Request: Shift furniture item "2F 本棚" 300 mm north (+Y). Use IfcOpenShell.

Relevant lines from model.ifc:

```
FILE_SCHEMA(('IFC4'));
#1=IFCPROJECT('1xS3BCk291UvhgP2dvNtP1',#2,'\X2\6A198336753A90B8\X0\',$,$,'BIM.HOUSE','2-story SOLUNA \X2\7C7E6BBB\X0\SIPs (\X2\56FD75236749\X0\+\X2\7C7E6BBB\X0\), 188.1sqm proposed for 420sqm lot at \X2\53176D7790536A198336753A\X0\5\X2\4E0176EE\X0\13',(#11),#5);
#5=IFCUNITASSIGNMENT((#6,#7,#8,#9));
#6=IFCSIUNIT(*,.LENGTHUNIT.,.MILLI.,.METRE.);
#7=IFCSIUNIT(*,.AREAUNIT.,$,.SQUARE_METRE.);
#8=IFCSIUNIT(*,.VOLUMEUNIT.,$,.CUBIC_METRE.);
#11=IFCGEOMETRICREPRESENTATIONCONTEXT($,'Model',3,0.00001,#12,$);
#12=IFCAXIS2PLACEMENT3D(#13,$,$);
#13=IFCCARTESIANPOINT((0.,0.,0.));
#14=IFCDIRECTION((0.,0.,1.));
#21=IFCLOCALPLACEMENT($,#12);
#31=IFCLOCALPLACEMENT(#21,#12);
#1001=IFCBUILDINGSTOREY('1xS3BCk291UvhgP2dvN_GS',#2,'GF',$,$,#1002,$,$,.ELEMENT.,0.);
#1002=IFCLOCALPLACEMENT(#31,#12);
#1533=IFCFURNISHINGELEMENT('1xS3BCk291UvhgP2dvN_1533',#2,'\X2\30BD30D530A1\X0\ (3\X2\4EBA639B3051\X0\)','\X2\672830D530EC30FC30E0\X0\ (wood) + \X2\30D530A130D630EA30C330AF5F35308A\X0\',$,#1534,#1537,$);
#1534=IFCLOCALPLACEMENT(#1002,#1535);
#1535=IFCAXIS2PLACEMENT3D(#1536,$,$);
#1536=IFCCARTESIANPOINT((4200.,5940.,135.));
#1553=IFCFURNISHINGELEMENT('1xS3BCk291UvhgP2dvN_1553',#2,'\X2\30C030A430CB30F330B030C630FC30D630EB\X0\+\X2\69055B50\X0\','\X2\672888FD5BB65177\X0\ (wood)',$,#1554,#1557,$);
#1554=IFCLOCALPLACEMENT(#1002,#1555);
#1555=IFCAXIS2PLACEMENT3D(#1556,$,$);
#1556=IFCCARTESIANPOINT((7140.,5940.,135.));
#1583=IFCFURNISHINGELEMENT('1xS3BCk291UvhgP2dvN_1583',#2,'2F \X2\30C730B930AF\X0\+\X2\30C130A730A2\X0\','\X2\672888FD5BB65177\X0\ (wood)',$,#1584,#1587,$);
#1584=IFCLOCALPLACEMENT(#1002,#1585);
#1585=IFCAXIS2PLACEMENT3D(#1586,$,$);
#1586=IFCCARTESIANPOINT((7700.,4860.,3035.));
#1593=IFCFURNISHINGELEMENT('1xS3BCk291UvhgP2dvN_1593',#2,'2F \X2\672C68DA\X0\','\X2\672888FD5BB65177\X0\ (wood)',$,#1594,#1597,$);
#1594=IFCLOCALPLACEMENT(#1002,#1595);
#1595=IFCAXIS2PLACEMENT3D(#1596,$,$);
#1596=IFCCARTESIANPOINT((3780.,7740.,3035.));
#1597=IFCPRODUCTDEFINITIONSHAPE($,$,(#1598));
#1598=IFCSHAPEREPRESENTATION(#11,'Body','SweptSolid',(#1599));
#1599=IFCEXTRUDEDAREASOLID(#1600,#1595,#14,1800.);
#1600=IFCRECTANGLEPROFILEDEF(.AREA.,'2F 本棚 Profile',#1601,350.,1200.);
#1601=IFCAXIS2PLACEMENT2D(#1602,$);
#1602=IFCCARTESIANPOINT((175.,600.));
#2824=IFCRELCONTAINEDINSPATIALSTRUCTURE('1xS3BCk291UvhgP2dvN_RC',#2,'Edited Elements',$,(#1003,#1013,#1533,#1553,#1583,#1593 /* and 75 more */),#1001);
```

```python
import ifcopenshell
import ifcopenshell.api.geometry
import ifcopenshell.util.placement

model = ifcopenshell.open("model.ifc")

item = model.by_guid("1xS3BCk291UvhgP2dvN_1593")
matrix = ifcopenshell.util.placement.get_local_placement(item.ObjectPlacement)
matrix[1, 3] += 300.0
ifcopenshell.api.geometry.edit_object_placement(model, product=item, matrix=matrix, is_si=False)

print(ifcopenshell.util.placement.get_local_placement(item.ObjectPlacement).round(3) + 0.0)

model.write("model_updated.ifc")
```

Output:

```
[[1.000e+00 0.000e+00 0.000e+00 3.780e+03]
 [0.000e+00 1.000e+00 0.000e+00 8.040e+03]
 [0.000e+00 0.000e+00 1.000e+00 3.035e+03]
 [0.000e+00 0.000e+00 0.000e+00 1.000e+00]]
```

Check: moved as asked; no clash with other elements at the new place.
